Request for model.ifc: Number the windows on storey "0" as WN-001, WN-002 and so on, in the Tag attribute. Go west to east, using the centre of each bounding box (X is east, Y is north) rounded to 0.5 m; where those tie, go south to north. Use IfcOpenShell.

First a look at what the model holds.

```python
import ifcopenshell
import ifcopenshell.util.element
import ifcopenshell.util.placement

model = ifcopenshell.open("model.ifc")
print(model.schema)
storey = next(s for s in model.by_type("IfcBuildingStorey") if s.Name == "0")
windows = [e for e in ifcopenshell.util.element.get_decomposition(storey) if e.is_a("IfcWindow")]
for e in sorted(windows, key=lambda e: e.id()):
    origin = ifcopenshell.util.placement.get_local_placement(e.ObjectPlacement)[:3, 3]
    print(e.id(), e.Tag, e.Name, origin.round(2) + 0.0, sep=" | ")
```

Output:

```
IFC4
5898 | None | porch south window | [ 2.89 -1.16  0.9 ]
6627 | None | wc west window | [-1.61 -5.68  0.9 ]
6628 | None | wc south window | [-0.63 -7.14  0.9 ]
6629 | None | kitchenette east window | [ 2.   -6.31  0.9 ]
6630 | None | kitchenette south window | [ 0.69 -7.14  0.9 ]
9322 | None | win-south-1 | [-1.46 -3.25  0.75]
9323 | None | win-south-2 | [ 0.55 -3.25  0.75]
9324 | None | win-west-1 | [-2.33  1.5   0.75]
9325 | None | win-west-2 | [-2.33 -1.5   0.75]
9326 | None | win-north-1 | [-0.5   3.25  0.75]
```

```python
import ifcopenshell
import ifcopenshell.geom
import ifcopenshell.util.element
import ifcopenshell.util.shape

model = ifcopenshell.open("model.ifc")
settings = ifcopenshell.geom.settings()
settings.set("use-world-coords", True)


def centre(element):
    shape = ifcopenshell.geom.create_shape(settings, element)
    return ifcopenshell.util.shape.get_bbox_centroid(shape.geometry)


storey = next(s for s in model.by_type("IfcBuildingStorey") if s.Name == "0")
windows = [e for e in ifcopenshell.util.element.get_decomposition(storey) if e.is_a("IfcWindow")]

# Insertion points can sit at a corner or the storey origin, so sort by the geometry (in metres).
centres = {e: centre(e) for e in windows}
windows.sort(key=lambda e: (round(centres[e][0] / 0.5), centres[e][1]))

for i, e in enumerate(windows, start=1):
    number = f"WN-0{i:02d}"
    e.Tag = number
    print(e.id(), number)

model.write("model_edited.ifc")
```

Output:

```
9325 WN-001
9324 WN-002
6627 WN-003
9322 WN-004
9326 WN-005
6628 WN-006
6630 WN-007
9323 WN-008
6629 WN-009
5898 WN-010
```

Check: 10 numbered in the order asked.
